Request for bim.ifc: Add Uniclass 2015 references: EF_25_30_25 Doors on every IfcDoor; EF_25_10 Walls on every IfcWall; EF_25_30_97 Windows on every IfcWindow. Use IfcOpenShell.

First a look at what the model holds.

```python
import ifcopenshell

model = ifcopenshell.open("bim.ifc")
print(model.schema)
print("classifications:", [c.Name for c in model.by_type("IfcClassification")])
for ifc_class in ("IfcDoor", "IfcRoof", "IfcStair", "IfcWall", "IfcWindow"):
    print(ifc_class, len(model.by_type(ifc_class)))
```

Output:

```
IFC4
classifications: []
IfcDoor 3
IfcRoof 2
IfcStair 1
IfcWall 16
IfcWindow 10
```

```python
import ifcopenshell
import ifcopenshell.api.classification

model = ifcopenshell.open("bim.ifc")

system = ifcopenshell.api.classification.add_classification(model, classification="Uniclass 2015")

codes = {
    "IfcDoor": ("EF_25_30_25", "Doors"),
    "IfcWall": ("EF_25_10", "Walls"),
    "IfcWindow": ("EF_25_30_97", "Windows"),
}
for ifc_class, (code, name) in codes.items():
    products = model.by_type(ifc_class)
    ifcopenshell.api.classification.add_reference(
        model, products=products, classification=system, identification=code, name=name
    )
    print(code, len(products))

model.write("bim_edited.ifc")
```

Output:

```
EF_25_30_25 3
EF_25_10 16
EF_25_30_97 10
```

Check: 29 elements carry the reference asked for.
